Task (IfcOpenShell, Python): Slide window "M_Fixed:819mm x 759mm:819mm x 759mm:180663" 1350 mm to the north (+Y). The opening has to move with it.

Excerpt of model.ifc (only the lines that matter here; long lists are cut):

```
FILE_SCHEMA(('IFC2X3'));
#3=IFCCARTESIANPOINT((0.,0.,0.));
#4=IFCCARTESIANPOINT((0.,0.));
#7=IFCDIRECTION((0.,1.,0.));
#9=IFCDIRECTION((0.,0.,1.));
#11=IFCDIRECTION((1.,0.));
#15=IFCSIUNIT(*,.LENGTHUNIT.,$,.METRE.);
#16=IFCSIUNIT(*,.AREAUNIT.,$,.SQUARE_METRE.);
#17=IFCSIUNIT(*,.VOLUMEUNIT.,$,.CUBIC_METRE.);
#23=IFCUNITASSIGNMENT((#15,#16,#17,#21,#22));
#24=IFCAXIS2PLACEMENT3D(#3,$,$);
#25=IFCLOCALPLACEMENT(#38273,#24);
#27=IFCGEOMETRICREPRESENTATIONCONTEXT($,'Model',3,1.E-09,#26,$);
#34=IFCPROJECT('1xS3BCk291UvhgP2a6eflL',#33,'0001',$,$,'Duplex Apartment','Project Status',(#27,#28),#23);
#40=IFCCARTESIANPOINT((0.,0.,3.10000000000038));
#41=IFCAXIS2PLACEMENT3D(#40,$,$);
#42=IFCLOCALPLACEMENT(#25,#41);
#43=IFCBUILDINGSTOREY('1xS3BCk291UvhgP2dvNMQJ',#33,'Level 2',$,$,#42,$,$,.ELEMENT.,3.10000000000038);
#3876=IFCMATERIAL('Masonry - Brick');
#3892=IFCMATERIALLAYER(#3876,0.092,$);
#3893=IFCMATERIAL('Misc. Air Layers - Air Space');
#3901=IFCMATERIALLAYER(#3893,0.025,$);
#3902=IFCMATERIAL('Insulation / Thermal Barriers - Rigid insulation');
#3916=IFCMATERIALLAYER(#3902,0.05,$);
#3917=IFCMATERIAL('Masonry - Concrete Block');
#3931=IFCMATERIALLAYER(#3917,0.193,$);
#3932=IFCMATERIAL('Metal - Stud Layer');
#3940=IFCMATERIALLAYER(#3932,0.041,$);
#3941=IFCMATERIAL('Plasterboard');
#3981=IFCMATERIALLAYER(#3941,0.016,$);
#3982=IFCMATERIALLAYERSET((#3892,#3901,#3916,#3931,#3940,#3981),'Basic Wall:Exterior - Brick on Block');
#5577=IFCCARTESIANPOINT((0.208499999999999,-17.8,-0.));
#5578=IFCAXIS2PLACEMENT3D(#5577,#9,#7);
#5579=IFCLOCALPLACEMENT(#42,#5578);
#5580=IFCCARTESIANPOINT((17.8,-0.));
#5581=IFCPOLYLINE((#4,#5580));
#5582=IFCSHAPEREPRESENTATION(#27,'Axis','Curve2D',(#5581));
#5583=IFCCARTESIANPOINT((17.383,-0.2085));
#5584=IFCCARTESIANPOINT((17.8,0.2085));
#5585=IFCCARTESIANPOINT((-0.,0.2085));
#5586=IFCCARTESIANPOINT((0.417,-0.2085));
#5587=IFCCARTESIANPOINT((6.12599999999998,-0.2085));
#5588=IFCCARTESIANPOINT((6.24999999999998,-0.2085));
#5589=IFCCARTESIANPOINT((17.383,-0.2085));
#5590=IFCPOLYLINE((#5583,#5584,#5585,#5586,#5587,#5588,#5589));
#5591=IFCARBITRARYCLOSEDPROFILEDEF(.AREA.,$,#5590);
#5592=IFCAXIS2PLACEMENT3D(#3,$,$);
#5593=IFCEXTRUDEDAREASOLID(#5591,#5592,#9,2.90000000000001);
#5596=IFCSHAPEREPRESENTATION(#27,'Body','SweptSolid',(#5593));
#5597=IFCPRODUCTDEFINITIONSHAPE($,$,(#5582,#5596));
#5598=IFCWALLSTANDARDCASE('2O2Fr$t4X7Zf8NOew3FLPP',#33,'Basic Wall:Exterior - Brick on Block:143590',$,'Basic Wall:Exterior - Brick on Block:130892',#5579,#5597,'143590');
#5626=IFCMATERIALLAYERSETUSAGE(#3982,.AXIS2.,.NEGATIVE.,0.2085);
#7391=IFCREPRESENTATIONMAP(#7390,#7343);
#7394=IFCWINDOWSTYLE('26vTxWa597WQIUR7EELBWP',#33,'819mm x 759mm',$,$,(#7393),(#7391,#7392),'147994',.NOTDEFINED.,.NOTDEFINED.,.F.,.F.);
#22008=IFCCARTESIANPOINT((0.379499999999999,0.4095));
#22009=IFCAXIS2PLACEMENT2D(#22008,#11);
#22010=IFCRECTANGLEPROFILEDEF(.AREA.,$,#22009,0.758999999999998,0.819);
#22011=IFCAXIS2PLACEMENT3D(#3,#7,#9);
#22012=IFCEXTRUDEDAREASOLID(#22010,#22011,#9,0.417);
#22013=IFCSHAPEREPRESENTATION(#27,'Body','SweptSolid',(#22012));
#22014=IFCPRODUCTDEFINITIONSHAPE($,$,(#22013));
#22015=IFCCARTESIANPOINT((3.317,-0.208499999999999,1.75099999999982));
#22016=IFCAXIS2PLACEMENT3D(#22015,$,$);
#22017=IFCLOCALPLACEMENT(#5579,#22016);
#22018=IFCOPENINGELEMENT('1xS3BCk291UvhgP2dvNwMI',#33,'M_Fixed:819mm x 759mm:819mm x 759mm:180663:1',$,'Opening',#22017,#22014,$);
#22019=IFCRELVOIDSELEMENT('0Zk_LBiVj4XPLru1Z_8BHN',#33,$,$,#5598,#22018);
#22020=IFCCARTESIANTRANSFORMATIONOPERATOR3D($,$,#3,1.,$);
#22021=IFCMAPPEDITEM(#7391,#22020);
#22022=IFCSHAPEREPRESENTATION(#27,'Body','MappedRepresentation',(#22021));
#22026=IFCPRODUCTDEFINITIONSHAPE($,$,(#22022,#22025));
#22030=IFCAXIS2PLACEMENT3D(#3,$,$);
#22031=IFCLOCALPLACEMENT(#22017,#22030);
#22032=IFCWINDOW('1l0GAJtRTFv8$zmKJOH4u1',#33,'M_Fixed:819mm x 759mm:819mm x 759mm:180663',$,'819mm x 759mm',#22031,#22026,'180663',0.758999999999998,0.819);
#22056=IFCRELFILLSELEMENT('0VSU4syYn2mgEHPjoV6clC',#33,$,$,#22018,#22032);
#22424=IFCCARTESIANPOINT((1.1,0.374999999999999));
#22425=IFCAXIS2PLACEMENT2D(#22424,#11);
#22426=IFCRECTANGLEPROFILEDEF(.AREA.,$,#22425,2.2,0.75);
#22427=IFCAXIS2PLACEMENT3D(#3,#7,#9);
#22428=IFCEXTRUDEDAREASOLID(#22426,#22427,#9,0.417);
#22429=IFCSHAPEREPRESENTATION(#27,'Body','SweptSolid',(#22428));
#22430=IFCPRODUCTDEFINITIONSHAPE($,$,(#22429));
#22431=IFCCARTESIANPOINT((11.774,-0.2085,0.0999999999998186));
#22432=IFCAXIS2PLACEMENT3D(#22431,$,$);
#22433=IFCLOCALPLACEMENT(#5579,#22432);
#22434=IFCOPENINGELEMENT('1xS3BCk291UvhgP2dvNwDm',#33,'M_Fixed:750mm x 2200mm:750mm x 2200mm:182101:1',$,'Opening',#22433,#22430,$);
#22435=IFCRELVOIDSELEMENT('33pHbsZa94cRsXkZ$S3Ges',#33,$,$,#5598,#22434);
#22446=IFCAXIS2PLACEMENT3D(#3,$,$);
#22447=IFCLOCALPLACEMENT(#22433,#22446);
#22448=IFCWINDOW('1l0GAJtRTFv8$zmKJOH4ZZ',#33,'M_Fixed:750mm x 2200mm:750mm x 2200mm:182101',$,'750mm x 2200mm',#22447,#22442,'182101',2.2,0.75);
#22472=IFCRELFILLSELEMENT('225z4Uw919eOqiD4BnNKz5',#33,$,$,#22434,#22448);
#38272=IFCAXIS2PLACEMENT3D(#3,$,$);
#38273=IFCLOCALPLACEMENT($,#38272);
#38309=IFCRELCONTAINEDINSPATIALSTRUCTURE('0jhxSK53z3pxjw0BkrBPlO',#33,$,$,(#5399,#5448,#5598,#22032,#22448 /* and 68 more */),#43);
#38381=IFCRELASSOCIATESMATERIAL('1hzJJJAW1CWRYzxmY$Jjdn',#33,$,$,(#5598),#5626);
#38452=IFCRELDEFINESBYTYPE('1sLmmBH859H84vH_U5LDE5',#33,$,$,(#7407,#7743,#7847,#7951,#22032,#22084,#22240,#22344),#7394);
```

```python
import ifcopenshell
import ifcopenshell.api.geometry
import ifcopenshell.util.placement
import ifcopenshell.util.unit

model = ifcopenshell.open("model.ifc")
unit_scale = ifcopenshell.util.unit.calculate_unit_scale(model)

window = model.by_guid("1l0GAJtRTFv8$zmKJOH4u1")
opening = window.FillsVoids[0].RelatingOpeningElement
wall = opening.VoidsElements[0].RelatingBuildingElement

wall_matrix = ifcopenshell.util.placement.get_local_placement(wall.ObjectPlacement)
shift = wall_matrix[:3, 0] * 1.35 / unit_scale
before = ifcopenshell.util.placement.get_local_placement(window.ObjectPlacement)[:3, 3].copy()

# The window is placed relative to its opening, so it follows when the opening moves.
matrix = ifcopenshell.util.placement.get_local_placement(opening.ObjectPlacement)
matrix[:3, 3] += shift
ifcopenshell.api.geometry.edit_object_placement(
    model, product=opening, matrix=matrix, is_si=False, should_transform_children=True
)

after = ifcopenshell.util.placement.get_local_placement(window.ObjectPlacement)[:3, 3]
print("window moved by", (after - before).round(3) + 0.0)

model.write("model_rev.ifc")
```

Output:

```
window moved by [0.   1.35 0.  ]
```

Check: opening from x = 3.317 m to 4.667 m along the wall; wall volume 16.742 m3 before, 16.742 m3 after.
